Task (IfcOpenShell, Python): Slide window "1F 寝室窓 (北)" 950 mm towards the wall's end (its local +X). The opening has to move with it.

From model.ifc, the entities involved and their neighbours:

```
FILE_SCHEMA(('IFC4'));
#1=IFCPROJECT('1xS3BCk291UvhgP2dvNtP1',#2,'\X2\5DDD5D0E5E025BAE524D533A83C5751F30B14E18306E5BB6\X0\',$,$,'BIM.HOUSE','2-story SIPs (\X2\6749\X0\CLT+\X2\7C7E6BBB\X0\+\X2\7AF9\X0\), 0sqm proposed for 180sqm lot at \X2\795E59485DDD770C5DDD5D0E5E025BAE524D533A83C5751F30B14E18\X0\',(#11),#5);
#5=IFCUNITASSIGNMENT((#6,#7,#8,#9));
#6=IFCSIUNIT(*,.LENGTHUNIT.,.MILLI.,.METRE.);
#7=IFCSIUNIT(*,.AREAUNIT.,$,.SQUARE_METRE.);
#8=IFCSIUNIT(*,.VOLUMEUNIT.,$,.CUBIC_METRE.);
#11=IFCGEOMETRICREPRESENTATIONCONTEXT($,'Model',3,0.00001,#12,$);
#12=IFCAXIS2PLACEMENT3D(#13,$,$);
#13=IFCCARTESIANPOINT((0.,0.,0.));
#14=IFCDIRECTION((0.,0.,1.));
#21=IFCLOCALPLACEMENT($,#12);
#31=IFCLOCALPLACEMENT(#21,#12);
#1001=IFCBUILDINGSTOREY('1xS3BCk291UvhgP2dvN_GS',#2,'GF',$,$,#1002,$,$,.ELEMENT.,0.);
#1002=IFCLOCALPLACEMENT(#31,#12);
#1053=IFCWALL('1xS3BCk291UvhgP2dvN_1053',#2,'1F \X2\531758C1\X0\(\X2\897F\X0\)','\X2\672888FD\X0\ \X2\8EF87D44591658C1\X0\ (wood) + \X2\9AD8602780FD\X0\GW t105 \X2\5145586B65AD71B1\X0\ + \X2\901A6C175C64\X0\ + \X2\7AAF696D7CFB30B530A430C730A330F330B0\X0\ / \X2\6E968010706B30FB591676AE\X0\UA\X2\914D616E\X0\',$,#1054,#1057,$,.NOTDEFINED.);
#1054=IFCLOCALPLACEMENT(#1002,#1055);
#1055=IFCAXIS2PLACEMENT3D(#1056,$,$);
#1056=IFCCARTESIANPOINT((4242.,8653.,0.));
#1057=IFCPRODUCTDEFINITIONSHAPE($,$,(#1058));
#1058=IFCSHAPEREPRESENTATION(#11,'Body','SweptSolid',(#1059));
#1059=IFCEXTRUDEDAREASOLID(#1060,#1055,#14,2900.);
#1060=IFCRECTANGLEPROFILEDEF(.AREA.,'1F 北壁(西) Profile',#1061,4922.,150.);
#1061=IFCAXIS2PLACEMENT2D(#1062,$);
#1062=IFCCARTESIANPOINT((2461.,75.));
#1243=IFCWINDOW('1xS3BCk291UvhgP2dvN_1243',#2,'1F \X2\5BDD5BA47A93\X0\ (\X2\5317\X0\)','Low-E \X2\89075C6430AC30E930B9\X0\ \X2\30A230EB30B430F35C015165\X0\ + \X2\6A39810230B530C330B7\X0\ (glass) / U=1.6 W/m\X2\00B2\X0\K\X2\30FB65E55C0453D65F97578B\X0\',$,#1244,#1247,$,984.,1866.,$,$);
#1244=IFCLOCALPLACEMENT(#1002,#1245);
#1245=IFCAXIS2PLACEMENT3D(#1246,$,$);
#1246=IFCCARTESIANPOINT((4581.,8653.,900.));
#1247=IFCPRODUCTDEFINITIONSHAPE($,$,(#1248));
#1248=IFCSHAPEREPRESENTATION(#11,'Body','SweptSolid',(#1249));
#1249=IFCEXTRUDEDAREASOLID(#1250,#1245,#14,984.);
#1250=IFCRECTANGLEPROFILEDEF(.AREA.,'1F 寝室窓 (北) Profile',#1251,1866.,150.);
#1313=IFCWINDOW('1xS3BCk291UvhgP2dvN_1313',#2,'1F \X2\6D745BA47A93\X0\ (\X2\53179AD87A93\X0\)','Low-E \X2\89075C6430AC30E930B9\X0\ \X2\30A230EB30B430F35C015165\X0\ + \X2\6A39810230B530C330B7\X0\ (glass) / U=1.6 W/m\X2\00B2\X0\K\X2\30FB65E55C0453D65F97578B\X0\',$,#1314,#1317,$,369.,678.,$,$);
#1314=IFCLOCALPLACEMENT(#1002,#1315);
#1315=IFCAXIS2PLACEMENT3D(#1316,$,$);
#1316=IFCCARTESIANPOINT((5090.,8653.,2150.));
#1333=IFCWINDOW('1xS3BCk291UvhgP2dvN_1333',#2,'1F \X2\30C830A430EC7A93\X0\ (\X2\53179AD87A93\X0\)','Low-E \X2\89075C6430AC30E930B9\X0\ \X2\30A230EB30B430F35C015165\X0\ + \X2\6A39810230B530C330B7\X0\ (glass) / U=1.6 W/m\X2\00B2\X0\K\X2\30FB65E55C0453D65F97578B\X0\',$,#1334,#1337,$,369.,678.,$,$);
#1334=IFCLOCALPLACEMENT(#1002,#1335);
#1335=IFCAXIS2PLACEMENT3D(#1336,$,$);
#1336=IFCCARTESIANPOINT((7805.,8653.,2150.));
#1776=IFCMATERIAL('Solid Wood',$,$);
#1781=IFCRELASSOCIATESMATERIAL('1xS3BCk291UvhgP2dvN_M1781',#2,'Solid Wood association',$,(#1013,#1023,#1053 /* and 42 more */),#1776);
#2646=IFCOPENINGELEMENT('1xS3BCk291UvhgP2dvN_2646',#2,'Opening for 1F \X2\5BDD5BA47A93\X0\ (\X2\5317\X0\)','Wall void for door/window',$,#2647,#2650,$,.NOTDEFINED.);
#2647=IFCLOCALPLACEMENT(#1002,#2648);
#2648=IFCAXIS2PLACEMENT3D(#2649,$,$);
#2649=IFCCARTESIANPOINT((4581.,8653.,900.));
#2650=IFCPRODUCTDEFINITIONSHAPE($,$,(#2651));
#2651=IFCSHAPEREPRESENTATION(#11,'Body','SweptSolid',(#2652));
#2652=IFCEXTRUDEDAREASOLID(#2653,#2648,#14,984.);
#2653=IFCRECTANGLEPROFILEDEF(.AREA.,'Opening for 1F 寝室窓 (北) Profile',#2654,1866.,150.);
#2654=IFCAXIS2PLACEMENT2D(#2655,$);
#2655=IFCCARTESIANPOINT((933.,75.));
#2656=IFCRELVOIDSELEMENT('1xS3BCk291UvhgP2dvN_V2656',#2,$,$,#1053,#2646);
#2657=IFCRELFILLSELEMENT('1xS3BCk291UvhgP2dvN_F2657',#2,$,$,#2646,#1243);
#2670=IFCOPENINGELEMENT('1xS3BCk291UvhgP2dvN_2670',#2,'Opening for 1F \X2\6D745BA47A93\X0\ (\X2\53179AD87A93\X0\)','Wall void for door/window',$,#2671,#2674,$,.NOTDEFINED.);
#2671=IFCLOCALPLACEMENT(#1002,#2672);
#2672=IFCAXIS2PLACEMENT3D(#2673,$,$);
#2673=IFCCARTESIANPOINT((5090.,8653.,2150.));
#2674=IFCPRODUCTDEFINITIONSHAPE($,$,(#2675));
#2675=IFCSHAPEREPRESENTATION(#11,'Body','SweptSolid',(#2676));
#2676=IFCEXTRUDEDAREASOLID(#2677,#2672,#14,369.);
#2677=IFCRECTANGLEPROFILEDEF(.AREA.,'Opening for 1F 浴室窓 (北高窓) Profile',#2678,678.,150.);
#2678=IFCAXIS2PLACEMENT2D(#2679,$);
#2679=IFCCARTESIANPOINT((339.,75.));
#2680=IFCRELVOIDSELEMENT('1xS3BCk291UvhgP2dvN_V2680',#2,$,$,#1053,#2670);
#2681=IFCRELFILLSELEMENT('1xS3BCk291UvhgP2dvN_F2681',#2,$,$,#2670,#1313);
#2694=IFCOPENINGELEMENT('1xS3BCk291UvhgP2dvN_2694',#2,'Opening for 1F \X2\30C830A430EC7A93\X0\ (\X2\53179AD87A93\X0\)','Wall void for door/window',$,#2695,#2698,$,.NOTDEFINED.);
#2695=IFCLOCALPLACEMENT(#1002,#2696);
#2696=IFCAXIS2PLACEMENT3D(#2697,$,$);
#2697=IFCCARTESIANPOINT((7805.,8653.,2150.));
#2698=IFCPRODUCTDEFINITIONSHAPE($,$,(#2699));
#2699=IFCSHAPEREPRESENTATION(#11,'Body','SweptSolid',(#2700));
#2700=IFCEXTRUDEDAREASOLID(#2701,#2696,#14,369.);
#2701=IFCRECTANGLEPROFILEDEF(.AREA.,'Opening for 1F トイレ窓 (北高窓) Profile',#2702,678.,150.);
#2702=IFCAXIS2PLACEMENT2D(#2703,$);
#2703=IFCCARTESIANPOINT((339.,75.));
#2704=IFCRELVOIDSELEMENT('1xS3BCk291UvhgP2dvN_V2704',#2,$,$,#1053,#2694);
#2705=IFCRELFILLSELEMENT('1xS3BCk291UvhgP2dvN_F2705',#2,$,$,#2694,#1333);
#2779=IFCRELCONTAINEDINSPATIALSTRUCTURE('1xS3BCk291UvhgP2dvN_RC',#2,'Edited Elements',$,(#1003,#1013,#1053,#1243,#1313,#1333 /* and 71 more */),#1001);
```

```python
import ifcopenshell
import ifcopenshell.api.geometry
import ifcopenshell.util.placement

model = ifcopenshell.open("model.ifc")

window = model.by_guid("1xS3BCk291UvhgP2dvN_1243")
opening = window.FillsVoids[0].RelatingOpeningElement
wall = opening.VoidsElements[0].RelatingBuildingElement

wall_matrix = ifcopenshell.util.placement.get_local_placement(wall.ObjectPlacement)
shift = wall_matrix[:3, 0] * 950.0
before = ifcopenshell.util.placement.get_local_placement(window.ObjectPlacement)[:3, 3].copy()

# The window is not placed relative to its opening, so move both.
for product in (opening, window):
    matrix = ifcopenshell.util.placement.get_local_placement(product.ObjectPlacement)
    matrix[:3, 3] += shift
    ifcopenshell.api.geometry.edit_object_placement(model, product=product, matrix=matrix, is_si=False)

after = ifcopenshell.util.placement.get_local_placement(window.ObjectPlacement)[:3, 3]
print("window moved by", (after - before).round(3) + 0.0)

model.write("model_updated.ifc")
```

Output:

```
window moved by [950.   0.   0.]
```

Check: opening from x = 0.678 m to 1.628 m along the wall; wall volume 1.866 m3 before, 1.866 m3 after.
